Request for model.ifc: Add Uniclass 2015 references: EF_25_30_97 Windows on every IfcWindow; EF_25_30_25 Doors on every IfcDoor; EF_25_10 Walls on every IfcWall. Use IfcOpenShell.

First a look at what the model holds.

```python
import ifcopenshell

model = ifcopenshell.open("model.ifc")
print(model.schema)
print("classifications:", [c.Name for c in model.by_type("IfcClassification")])
for ifc_class in ("IfcDoor", "IfcRoof", "IfcStair", "IfcWall", "IfcWindow"):
    print(ifc_class, len(model.by_type(ifc_class)))
```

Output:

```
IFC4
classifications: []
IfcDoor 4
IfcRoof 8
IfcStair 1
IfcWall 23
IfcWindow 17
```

```python
import ifcopenshell
import ifcopenshell.api.classification

model = ifcopenshell.open("model.ifc")

system = ifcopenshell.api.classification.add_classification(model, classification="Uniclass 2015")

codes = {
    "IfcWindow": ("EF_25_30_97", "Windows"),
    "IfcDoor": ("EF_25_30_25", "Doors"),
    "IfcWall": ("EF_25_10", "Walls"),
}
for ifc_class, (code, name) in codes.items():
    products = model.by_type(ifc_class)
    ifcopenshell.api.classification.add_reference(
        model, products=products, classification=system, identification=code, name=name
    )
    print(code, len(products))

model.write("model_updated.ifc")
```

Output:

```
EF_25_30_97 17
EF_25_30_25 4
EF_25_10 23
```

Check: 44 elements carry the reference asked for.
